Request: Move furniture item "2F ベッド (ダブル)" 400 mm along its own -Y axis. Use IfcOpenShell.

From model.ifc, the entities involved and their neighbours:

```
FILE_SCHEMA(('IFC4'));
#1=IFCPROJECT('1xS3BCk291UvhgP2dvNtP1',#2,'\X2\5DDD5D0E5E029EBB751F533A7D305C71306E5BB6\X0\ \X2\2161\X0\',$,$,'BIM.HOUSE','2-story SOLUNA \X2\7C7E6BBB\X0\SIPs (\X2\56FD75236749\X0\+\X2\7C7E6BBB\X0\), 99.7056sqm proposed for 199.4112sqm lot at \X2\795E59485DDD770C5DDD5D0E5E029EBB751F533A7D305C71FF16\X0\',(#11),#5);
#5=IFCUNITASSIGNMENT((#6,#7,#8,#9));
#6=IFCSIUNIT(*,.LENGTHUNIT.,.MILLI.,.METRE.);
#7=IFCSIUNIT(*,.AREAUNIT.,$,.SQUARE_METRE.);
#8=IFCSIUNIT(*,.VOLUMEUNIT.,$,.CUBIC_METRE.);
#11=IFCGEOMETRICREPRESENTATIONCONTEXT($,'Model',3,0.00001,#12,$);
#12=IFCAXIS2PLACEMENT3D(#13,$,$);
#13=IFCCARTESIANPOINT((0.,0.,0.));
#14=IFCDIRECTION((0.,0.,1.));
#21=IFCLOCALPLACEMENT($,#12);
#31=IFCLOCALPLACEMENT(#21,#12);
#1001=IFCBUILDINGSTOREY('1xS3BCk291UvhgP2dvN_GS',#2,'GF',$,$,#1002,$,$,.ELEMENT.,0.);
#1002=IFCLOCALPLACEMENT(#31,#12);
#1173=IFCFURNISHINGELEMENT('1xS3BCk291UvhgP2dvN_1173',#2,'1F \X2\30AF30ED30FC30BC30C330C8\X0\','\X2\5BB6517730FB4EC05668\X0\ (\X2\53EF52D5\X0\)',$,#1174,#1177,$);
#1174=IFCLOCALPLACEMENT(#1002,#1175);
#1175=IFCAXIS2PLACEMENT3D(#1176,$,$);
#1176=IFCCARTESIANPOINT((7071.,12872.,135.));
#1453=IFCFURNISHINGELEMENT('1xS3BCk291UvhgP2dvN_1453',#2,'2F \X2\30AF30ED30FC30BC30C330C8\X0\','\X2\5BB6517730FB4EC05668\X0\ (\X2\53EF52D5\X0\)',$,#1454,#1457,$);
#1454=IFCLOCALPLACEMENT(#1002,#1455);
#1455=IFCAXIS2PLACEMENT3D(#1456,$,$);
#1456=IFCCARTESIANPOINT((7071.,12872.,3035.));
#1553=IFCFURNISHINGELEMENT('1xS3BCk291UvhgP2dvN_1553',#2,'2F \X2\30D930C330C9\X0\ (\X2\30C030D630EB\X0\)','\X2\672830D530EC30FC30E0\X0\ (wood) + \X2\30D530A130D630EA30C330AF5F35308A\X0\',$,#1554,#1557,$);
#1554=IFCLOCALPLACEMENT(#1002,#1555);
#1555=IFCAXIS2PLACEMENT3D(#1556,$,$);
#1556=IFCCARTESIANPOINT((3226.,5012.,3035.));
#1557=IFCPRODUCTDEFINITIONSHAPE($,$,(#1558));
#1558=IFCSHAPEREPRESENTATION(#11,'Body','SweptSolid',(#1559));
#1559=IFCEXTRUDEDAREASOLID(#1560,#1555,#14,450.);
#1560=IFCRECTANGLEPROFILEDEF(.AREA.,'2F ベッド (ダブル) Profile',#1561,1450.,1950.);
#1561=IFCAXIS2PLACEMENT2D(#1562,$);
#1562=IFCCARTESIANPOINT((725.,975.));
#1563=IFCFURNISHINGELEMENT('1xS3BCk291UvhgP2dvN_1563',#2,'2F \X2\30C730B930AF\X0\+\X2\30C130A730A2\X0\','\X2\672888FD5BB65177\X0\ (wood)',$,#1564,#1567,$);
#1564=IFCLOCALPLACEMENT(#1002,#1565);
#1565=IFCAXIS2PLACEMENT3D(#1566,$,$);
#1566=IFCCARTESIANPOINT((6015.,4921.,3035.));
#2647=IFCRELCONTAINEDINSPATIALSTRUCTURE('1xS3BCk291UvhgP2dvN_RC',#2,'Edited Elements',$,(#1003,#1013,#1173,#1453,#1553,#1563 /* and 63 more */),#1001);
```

```python
import ifcopenshell
import ifcopenshell.api.geometry
import ifcopenshell.util.placement
import ifcopenshell.util.unit

model = ifcopenshell.open("model.ifc")
unit_scale = ifcopenshell.util.unit.calculate_unit_scale(model)

item = model.by_guid("1xS3BCk291UvhgP2dvN_1553")
matrix = ifcopenshell.util.placement.get_local_placement(item.ObjectPlacement)
matrix[:3, 3] -= matrix[:3, 1] * 0.4 / unit_scale
ifcopenshell.api.geometry.edit_object_placement(model, product=item, matrix=matrix, is_si=False)

print(ifcopenshell.util.placement.get_local_placement(item.ObjectPlacement).round(3) + 0.0)

model.write("model_rev.ifc")
```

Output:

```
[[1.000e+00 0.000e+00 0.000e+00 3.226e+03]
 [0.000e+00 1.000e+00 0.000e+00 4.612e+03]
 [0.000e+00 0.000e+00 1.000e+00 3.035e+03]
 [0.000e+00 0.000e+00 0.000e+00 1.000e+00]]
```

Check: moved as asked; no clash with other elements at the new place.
